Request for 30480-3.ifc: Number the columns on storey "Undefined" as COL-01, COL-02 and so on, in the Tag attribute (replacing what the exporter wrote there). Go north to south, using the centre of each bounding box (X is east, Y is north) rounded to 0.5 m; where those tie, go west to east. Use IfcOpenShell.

First a look at what the model holds.

```python
import ifcopenshell
import ifcopenshell.util.element
import ifcopenshell.util.placement

model = ifcopenshell.open("30480-3.ifc")
print(model.schema)
storey = next(s for s in model.by_type("IfcBuildingStorey") if s.Name == "Undefined")
columns = [e for e in ifcopenshell.util.element.get_decomposition(storey) if e.is_a("IfcColumn")]
for e in sorted(columns, key=lambda e: e.id()):
    origin = ifcopenshell.util.placement.get_local_placement(e.ObjectPlacement)[:3, 3]
    print(e.id(), e.Tag, e.Name, origin.round(2) + 0.0, sep=" | ")
```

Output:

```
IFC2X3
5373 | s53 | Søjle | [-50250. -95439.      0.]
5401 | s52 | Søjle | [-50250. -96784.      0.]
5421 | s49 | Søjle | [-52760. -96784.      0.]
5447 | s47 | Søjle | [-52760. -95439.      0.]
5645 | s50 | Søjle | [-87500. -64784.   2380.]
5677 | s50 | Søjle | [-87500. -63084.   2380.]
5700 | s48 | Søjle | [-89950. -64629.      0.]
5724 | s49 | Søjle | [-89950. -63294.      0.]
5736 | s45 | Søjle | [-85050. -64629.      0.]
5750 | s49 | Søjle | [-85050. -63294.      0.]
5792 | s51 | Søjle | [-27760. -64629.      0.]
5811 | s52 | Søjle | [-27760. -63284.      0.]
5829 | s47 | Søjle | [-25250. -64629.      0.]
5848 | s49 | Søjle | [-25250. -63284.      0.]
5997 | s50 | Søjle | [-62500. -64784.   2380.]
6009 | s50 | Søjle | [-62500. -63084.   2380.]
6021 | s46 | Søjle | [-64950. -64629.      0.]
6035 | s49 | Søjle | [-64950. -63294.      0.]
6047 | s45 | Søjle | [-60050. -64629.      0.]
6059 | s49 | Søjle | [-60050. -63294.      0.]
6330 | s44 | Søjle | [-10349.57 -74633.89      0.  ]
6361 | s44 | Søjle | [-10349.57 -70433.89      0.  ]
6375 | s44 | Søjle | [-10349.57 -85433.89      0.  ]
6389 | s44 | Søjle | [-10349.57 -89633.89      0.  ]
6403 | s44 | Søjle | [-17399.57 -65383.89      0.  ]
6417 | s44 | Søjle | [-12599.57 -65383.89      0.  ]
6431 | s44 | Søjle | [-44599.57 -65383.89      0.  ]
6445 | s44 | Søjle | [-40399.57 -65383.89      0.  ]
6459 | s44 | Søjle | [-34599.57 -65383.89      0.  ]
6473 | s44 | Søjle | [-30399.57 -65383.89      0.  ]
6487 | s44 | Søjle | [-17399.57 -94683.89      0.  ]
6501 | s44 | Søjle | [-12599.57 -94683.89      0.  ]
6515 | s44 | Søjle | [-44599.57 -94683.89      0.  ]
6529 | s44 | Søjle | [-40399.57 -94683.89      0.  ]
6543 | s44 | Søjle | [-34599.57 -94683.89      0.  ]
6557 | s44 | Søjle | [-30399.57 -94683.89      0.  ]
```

```python
import ifcopenshell
import ifcopenshell.geom
import ifcopenshell.util.element
import ifcopenshell.util.shape

model = ifcopenshell.open("30480-3.ifc")
settings = ifcopenshell.geom.settings()
settings.set("use-world-coords", True)


def centre(element):
    shape = ifcopenshell.geom.create_shape(settings, element)
    return ifcopenshell.util.shape.get_bbox_centroid(shape.geometry)


storey = next(s for s in model.by_type("IfcBuildingStorey") if s.Name == "Undefined")
columns = [e for e in ifcopenshell.util.element.get_decomposition(storey) if e.is_a("IfcColumn")]

# Insertion points can sit at a corner or the storey origin, so sort by the geometry (in metres).
centres = {e: centre(e) for e in columns}
columns.sort(key=lambda e: (-round(centres[e][1] / 0.5), centres[e][0]))

for i, e in enumerate(columns, start=1):
    number = f"COL-{i:02d}"
    e.Tag = number
    print(e.id(), number)

model.write("30480-3_edited.ifc")
```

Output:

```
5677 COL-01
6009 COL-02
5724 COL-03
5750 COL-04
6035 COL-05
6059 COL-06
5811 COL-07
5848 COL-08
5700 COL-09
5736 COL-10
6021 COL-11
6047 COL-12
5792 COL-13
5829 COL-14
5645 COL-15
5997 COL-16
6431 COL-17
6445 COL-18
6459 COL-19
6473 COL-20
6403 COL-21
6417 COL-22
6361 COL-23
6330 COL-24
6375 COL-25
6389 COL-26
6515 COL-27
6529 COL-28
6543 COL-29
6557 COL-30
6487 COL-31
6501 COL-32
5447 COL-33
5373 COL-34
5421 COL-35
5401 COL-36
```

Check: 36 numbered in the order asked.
